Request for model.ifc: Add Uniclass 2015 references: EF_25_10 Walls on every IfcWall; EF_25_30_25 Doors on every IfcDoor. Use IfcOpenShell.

First a look at what the model holds.

```python
import ifcopenshell

model = ifcopenshell.open("model.ifc")
print(model.schema)
print("classifications:", [c.Name for c in model.by_type("IfcClassification")])
for ifc_class in ("IfcDoor", "IfcRoof", "IfcStair", "IfcWall", "IfcWindow"):
    print(ifc_class, len(model.by_type(ifc_class)))
```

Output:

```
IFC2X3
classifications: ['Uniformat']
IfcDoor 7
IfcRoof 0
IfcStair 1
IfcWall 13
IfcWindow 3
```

```python
import ifcopenshell
import ifcopenshell.api.classification

model = ifcopenshell.open("model.ifc")

# IFC2X3 requires Source and Edition and has no link from the project to the system.
system = model.create_entity("IfcClassification", Source="NBS", Edition="2015", Name="Uniclass 2015")

codes = {
    "IfcWall": ("EF_25_10", "Walls"),
    "IfcDoor": ("EF_25_30_25", "Doors"),
}
for ifc_class, (code, name) in codes.items():
    products = model.by_type(ifc_class)
    ifcopenshell.api.classification.add_reference(
        model, products=products, classification=system, identification=code, name=name
    )
    print(code, len(products))

model.write("model_updated.ifc")
```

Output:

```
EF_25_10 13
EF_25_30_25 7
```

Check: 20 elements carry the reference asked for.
